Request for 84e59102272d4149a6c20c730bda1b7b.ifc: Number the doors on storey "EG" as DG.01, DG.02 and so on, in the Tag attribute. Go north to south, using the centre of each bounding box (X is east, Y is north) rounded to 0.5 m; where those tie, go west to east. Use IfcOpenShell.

First a look at what the model holds.

```python
import ifcopenshell
import ifcopenshell.util.element
import ifcopenshell.util.placement

model = ifcopenshell.open("84e59102272d4149a6c20c730bda1b7b.ifc")
print(model.schema)
storey = next(s for s in model.by_type("IfcBuildingStorey") if s.Name == "EG")
doors = [e for e in ifcopenshell.util.element.get_decomposition(storey) if e.is_a("IfcDoor")]
for e in sorted(doors, key=lambda e: e.id()):
    origin = ifcopenshell.util.placement.get_local_placement(e.ObjectPlacement)[:3, 3]
    print(e.id(), e.Tag, e.Name, origin.round(2) + 0.0, sep=" | ")
```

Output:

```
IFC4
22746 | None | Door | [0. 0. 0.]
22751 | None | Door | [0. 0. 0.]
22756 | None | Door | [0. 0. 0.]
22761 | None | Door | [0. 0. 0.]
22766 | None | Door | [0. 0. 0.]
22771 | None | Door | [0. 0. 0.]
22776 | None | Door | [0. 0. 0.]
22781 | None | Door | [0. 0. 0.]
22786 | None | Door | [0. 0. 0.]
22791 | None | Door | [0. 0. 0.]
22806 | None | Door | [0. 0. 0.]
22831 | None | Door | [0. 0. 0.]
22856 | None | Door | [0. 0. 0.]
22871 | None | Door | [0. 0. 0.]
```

```python
import ifcopenshell
import ifcopenshell.geom
import ifcopenshell.util.element
import ifcopenshell.util.shape

model = ifcopenshell.open("84e59102272d4149a6c20c730bda1b7b.ifc")
settings = ifcopenshell.geom.settings()
settings.set("use-world-coords", True)


def centre(element):
    shape = ifcopenshell.geom.create_shape(settings, element)
    return ifcopenshell.util.shape.get_bbox_centroid(shape.geometry)


storey = next(s for s in model.by_type("IfcBuildingStorey") if s.Name == "EG")
doors = [e for e in ifcopenshell.util.element.get_decomposition(storey) if e.is_a("IfcDoor")]

# Insertion points can sit at a corner or the storey origin, so sort by the geometry (in metres).
centres = {e: centre(e) for e in doors}
doors.sort(key=lambda e: (-round(centres[e][1] / 0.5), centres[e][0]))

for i, e in enumerate(doors, start=1):
    number = f"DG.{i:02d}"
    e.Tag = number
    print(e.id(), number)

model.write("84e59102272d4149a6c20c730bda1b7b_updated.ifc")
```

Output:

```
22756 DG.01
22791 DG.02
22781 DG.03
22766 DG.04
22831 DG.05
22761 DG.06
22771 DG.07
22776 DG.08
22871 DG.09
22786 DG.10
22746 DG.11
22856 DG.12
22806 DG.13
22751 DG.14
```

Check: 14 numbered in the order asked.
